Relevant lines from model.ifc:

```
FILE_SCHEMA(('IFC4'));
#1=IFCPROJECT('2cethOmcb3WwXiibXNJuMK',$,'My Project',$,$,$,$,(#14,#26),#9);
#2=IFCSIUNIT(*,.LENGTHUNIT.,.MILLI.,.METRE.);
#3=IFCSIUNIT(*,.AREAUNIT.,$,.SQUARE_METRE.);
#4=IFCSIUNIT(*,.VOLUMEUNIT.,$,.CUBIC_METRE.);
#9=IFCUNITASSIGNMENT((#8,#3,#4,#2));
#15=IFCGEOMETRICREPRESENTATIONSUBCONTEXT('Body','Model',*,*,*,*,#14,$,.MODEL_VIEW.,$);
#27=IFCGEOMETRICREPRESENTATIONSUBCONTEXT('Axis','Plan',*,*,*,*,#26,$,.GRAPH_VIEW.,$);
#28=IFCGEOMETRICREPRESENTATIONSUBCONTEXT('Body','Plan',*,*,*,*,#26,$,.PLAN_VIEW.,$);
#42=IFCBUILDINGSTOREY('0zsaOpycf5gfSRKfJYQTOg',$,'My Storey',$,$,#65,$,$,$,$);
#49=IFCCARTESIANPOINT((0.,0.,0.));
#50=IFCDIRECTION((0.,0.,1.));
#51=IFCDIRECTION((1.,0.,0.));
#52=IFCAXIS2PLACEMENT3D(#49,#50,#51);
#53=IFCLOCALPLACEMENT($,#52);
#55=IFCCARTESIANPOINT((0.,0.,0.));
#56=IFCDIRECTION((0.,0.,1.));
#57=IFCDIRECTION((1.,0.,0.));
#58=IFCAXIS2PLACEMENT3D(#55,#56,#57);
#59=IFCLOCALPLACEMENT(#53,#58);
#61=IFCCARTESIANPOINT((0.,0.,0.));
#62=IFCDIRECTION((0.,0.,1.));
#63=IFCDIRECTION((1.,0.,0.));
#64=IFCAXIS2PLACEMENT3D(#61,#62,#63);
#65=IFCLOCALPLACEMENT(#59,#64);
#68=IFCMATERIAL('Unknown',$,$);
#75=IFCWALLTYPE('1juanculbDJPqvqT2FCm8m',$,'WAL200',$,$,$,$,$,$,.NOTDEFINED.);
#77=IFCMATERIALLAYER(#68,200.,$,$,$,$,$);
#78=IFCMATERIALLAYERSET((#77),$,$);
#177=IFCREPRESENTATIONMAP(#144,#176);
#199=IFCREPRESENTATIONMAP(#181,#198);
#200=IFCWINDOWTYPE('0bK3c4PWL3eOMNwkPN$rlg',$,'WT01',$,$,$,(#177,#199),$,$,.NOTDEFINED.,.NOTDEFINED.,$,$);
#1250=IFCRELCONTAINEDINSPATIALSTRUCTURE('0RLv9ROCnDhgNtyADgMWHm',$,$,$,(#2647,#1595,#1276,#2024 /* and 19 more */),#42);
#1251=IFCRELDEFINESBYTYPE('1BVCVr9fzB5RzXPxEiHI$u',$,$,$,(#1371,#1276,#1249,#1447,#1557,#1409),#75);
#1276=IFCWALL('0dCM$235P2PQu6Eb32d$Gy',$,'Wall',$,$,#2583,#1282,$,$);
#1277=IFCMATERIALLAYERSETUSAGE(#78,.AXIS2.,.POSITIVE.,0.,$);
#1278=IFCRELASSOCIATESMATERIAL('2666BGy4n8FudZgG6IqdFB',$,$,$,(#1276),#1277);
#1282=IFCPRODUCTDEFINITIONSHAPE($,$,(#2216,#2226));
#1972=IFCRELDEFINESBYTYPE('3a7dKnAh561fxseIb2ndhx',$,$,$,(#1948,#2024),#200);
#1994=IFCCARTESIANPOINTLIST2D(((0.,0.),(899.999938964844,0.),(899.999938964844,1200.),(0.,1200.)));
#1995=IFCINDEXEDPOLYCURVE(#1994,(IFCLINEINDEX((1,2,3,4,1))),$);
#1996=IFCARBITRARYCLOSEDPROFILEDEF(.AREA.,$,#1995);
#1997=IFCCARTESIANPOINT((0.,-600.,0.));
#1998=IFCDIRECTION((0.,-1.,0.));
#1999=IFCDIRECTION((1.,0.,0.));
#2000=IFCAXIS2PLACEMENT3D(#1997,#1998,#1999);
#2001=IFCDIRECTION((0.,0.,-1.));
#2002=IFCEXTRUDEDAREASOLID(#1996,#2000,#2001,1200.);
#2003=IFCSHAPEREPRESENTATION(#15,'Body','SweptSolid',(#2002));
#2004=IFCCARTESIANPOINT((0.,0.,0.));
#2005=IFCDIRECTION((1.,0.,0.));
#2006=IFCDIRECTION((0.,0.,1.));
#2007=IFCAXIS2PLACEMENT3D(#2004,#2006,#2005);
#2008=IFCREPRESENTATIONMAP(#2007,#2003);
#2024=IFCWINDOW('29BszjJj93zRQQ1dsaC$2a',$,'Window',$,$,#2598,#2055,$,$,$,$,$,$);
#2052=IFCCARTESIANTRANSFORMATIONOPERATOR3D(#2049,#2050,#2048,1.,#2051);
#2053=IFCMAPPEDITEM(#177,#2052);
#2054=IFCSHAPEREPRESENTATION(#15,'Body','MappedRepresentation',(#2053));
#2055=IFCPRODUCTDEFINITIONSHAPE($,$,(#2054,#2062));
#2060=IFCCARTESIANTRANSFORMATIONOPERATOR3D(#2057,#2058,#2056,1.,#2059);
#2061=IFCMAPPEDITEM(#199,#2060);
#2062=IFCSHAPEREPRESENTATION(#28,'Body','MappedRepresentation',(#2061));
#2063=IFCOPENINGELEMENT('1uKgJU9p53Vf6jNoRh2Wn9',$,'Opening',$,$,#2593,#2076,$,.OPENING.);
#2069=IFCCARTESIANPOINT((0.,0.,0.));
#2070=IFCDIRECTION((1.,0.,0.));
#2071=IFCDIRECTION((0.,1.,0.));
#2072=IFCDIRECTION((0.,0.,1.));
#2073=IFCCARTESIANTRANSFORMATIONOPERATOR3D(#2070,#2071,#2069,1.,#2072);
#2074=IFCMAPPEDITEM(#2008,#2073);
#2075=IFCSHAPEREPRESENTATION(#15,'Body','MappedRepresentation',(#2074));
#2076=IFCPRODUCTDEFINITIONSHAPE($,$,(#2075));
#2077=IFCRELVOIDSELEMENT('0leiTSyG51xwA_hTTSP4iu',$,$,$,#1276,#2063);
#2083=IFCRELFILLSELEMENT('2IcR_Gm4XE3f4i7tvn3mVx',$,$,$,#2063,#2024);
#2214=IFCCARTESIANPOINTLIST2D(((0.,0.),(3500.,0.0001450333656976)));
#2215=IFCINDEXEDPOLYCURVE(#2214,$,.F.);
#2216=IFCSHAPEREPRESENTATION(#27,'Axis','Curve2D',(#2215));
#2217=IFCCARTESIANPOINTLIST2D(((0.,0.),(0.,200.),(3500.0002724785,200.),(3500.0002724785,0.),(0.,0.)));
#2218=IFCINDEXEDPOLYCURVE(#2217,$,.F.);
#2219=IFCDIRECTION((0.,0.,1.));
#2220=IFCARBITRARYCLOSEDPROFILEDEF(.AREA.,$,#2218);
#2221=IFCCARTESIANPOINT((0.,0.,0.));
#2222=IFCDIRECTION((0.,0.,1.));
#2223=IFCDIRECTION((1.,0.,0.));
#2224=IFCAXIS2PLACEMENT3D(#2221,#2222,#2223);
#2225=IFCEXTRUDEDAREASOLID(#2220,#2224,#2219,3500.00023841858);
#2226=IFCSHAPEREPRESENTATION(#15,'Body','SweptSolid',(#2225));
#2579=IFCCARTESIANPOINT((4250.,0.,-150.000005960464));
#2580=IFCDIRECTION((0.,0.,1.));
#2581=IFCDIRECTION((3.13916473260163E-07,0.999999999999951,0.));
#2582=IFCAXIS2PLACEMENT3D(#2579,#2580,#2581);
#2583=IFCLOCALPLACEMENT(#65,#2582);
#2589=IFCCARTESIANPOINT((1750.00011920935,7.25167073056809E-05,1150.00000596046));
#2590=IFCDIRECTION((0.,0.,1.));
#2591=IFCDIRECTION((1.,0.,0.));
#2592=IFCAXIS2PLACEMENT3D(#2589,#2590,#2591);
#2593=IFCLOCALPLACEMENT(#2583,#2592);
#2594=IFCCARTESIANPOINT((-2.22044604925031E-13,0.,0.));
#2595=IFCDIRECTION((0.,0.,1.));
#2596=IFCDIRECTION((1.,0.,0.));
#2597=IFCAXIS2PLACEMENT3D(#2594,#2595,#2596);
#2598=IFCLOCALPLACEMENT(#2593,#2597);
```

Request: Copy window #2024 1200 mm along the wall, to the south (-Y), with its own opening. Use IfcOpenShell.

```python
import ifcopenshell
import ifcopenshell.api.feature
import ifcopenshell.api.geometry
import ifcopenshell.api.root
import ifcopenshell.geom
import ifcopenshell.util.element
import ifcopenshell.util.placement
import ifcopenshell.util.shape

model = ifcopenshell.open("model.ifc")
settings = ifcopenshell.geom.settings()


def volume(element):
    """Net volume in cubic metres, openings subtracted."""
    shape = ifcopenshell.geom.create_shape(settings, element)
    return ifcopenshell.util.shape.get_volume(shape.geometry)


window = model.by_guid("29BszjJj93zRQQ1dsaC$2a")
opening = window.FillsVoids[0].RelatingOpeningElement
wall = opening.VoidsElements[0].RelatingBuildingElement
before = volume(wall)
shift = ifcopenshell.util.placement.get_local_placement(wall.ObjectPlacement)[:3, 0] * -1200.0

# copy_class copies the void relationship, type, container and properties, but no geometry.
new_opening = ifcopenshell.api.root.copy_class(model, product=opening)
new_opening.Representation = ifcopenshell.util.element.copy_deep(
    model, opening.Representation, exclude=["IfcGeometricRepresentationContext", "IfcRepresentationMap"]
)
new_window = ifcopenshell.api.root.copy_class(model, product=window)
new_window.Representation = ifcopenshell.util.element.copy_deep(
    model, window.Representation, exclude=["IfcGeometricRepresentationContext", "IfcRepresentationMap"]
)
ifcopenshell.api.feature.add_filling(model, opening=new_opening, element=new_window)

for old, new in ((opening, new_opening), (window, new_window)):
    matrix = ifcopenshell.util.placement.get_local_placement(old.ObjectPlacement)
    matrix[:3, 3] += shift
    ifcopenshell.api.geometry.edit_object_placement(model, product=new, matrix=matrix, is_si=False)

after = volume(wall)

print(f"wall volume {before:.3f} -> {after:.3f} m3")

model.write("model_edited.ifc")
```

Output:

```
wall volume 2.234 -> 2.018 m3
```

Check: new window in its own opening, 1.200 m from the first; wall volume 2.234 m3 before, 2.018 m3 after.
